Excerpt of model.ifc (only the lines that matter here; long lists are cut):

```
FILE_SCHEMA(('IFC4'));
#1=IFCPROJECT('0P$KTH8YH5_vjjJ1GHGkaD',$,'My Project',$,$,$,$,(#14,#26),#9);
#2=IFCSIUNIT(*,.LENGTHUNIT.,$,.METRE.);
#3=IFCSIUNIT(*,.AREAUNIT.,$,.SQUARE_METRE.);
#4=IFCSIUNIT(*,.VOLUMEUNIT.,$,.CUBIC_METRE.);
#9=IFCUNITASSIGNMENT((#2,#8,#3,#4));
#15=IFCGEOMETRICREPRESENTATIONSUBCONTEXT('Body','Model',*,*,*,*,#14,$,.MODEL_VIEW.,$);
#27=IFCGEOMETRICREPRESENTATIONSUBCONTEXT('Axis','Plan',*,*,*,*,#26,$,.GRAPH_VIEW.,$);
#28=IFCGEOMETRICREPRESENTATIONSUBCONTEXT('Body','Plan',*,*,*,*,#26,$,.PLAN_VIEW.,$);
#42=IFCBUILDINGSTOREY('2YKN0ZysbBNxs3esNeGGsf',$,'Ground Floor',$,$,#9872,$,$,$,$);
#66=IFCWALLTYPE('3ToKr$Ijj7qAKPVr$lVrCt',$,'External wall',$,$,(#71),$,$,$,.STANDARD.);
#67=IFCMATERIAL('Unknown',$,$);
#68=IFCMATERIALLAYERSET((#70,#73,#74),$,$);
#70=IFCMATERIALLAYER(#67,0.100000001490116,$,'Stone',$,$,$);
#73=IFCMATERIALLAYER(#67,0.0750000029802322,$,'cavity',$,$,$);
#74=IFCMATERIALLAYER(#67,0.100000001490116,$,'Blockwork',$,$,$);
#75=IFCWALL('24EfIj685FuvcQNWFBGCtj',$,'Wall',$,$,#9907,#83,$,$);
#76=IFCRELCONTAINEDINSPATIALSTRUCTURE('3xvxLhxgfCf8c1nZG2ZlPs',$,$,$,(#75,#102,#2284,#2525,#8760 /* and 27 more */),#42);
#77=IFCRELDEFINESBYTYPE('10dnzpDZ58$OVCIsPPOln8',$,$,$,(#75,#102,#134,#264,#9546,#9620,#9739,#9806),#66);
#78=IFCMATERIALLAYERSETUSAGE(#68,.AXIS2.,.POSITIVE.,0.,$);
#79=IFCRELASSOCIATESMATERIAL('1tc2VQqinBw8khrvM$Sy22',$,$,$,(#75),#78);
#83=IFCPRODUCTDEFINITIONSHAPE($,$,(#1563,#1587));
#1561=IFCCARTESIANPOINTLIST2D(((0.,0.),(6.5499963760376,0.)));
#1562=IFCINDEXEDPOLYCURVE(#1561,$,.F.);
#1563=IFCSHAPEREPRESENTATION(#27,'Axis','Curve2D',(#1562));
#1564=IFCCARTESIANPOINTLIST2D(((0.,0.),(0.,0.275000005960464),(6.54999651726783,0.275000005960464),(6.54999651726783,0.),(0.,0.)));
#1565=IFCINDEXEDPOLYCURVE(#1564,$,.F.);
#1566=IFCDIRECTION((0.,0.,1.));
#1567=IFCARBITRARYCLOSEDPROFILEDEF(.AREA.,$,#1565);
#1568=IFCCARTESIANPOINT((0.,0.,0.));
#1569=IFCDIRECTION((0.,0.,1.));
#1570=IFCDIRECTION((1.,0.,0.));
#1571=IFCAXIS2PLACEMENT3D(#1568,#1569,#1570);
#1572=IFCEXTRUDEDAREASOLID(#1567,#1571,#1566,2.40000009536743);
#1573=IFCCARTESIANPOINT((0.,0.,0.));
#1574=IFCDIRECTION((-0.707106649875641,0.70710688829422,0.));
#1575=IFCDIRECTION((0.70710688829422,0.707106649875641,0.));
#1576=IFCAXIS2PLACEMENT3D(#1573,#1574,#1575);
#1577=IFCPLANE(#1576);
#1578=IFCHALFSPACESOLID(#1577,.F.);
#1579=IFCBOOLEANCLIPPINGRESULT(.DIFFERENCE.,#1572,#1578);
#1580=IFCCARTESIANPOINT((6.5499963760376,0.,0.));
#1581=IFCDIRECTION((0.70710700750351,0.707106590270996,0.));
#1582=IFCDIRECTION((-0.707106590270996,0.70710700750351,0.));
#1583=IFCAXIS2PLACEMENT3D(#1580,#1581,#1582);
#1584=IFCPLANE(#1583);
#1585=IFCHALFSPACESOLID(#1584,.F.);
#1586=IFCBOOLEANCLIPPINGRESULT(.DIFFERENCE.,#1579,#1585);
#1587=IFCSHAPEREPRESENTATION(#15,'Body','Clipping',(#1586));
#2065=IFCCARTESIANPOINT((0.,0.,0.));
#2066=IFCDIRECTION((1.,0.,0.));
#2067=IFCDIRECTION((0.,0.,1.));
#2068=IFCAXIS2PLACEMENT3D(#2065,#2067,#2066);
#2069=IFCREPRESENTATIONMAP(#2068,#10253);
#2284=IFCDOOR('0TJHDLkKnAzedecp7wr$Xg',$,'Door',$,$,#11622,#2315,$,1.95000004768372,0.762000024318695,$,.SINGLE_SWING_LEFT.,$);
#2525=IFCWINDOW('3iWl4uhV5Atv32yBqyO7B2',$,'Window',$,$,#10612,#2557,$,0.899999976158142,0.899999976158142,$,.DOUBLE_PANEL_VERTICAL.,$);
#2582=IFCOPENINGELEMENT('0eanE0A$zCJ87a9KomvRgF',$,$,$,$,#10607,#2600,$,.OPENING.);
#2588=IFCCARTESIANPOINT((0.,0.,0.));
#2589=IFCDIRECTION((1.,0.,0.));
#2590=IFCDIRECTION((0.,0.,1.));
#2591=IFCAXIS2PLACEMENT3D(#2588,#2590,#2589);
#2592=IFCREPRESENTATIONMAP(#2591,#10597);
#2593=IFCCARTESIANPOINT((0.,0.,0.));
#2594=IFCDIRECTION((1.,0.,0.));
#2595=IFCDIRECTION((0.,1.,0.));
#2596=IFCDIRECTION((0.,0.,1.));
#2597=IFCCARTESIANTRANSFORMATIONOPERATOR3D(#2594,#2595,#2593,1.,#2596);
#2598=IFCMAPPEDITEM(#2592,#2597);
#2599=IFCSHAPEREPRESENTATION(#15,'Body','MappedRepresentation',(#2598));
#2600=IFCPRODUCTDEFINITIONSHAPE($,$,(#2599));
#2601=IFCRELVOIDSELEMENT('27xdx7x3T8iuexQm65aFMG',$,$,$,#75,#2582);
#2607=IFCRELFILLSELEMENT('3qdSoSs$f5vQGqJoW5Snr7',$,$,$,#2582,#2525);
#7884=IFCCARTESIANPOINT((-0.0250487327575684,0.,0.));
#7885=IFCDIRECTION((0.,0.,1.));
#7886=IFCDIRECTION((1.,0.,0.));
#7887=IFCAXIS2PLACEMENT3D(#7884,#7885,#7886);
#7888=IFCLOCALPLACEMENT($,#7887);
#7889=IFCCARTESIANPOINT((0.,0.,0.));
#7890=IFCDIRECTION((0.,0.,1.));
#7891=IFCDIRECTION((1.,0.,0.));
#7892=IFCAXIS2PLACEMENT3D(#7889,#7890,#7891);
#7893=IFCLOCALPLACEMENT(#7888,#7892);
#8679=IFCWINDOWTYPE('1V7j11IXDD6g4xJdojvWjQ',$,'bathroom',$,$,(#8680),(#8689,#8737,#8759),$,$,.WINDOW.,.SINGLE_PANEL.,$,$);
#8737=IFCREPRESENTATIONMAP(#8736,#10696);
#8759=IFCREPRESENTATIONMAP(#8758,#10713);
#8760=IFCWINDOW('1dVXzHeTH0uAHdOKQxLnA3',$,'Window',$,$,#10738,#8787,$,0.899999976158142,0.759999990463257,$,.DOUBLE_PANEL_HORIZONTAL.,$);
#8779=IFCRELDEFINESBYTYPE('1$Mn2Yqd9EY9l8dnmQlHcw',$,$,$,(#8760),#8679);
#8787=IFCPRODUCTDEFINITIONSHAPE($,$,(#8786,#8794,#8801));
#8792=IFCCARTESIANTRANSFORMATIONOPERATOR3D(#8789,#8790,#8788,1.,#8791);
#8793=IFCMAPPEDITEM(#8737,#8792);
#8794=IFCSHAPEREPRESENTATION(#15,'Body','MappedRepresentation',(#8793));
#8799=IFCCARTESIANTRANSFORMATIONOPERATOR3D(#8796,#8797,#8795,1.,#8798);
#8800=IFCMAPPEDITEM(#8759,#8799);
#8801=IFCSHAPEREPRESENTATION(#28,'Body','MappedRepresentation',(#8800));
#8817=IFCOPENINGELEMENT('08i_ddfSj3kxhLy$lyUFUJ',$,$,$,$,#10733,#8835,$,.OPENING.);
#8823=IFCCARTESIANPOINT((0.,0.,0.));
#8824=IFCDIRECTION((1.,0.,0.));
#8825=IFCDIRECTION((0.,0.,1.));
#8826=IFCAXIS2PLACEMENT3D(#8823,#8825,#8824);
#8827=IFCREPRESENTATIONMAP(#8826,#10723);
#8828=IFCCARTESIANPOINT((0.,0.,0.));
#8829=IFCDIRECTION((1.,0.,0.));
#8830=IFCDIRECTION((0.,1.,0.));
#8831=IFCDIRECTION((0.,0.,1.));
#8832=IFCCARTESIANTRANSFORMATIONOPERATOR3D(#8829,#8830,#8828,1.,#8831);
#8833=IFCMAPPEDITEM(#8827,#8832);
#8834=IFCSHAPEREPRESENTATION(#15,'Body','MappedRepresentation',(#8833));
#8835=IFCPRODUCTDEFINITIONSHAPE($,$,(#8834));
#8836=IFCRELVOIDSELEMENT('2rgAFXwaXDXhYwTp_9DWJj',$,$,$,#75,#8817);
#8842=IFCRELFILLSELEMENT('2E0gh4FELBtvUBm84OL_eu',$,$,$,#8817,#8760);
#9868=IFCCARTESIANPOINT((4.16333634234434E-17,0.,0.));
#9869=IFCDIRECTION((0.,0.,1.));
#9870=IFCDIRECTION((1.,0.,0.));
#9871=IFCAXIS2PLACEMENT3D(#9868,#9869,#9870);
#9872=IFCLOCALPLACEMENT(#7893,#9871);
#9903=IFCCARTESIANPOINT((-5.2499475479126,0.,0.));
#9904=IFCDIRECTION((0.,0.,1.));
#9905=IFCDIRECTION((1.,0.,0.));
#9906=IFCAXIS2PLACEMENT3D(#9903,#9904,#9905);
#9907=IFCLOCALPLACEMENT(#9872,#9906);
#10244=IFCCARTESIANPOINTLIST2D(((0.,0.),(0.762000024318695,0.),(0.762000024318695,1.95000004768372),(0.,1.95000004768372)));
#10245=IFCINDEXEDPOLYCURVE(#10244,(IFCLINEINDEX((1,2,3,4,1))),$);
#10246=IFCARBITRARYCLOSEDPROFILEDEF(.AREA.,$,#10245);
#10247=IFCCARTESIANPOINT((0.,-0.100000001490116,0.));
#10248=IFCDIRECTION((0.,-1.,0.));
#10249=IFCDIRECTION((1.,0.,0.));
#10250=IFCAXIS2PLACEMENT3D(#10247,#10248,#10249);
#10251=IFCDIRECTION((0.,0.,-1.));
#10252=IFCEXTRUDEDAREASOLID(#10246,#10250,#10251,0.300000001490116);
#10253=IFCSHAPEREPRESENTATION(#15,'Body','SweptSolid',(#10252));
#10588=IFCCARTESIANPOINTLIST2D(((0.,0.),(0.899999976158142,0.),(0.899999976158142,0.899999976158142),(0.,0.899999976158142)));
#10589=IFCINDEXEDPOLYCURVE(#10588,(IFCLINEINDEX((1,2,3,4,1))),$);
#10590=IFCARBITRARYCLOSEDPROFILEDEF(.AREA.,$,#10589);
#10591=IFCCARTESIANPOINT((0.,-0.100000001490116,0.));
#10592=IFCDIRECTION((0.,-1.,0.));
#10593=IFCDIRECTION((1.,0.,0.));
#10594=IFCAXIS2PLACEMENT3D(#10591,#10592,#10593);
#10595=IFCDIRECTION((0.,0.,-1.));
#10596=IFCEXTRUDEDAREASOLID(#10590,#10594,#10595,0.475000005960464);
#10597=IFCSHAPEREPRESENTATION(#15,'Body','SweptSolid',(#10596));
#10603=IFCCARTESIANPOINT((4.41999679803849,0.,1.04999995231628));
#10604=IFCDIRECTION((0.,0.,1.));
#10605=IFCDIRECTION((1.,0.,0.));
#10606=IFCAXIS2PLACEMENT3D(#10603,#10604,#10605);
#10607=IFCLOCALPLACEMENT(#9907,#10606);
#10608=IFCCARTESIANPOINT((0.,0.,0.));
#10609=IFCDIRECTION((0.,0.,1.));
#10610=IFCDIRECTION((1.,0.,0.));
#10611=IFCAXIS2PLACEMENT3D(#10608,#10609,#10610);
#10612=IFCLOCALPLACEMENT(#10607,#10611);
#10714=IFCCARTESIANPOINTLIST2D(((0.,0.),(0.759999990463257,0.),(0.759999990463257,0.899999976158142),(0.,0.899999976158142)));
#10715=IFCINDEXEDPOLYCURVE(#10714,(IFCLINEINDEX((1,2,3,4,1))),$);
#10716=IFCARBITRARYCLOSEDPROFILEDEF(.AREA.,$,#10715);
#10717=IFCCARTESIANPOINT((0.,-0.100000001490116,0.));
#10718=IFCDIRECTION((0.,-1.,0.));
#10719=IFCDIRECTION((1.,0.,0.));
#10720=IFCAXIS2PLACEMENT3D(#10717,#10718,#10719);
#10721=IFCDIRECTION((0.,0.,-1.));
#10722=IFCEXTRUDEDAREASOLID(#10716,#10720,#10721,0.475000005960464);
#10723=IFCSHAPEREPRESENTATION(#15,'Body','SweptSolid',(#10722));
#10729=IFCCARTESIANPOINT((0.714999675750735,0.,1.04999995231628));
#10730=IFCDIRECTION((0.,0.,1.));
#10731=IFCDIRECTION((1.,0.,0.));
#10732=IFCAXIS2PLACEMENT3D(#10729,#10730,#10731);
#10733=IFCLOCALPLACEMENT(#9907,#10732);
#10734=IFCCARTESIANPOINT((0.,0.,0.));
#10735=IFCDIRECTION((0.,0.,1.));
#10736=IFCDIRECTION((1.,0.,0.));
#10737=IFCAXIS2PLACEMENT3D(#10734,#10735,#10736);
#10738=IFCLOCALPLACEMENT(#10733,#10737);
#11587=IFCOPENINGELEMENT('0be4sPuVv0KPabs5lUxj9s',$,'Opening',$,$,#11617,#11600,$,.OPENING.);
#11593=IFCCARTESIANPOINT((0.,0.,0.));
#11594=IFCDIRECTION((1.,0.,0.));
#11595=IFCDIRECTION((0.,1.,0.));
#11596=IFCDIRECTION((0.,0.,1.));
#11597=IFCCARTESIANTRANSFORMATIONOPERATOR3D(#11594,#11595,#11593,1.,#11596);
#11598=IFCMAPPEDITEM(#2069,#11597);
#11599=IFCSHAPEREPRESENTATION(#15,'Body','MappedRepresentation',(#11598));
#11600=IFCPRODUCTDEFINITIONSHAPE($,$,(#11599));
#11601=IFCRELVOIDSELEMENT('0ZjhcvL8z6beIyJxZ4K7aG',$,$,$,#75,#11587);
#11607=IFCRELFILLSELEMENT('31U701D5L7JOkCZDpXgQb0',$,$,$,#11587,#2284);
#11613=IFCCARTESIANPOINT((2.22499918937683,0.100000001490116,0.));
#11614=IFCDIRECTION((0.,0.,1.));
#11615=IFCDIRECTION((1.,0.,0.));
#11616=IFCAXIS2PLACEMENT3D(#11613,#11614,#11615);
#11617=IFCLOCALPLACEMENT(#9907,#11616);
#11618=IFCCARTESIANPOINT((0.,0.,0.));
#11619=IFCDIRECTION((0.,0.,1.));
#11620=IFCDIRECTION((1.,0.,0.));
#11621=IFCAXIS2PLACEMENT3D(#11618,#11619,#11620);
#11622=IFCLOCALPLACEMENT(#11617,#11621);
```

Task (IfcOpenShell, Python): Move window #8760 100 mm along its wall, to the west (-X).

```python
import ifcopenshell
import ifcopenshell.api.geometry
import ifcopenshell.util.placement

model = ifcopenshell.open("model.ifc")

window = model.by_guid("1dVXzHeTH0uAHdOKQxLnA3")
opening = window.FillsVoids[0].RelatingOpeningElement
wall = opening.VoidsElements[0].RelatingBuildingElement

wall_matrix = ifcopenshell.util.placement.get_local_placement(wall.ObjectPlacement)
shift = wall_matrix[:3, 0] * -0.1
before = ifcopenshell.util.placement.get_local_placement(window.ObjectPlacement)[:3, 3].copy()

# The window is placed relative to its opening, so it follows when the opening moves.
matrix = ifcopenshell.util.placement.get_local_placement(opening.ObjectPlacement)
matrix[:3, 3] += shift
ifcopenshell.api.geometry.edit_object_placement(
    model, product=opening, matrix=matrix, is_si=False, should_transform_children=True
)

after = ifcopenshell.util.placement.get_local_placement(window.ObjectPlacement)[:3, 3]
print("window moved by", (after - before).round(3) + 0.0)

model.write("model_v2.ifc")
```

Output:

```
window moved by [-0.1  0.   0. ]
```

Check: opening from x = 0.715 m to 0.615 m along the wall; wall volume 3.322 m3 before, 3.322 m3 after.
